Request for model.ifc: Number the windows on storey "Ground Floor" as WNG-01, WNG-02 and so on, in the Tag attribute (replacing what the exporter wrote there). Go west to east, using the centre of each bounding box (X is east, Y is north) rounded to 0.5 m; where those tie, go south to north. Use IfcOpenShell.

First a look at what the model holds.

```python
import ifcopenshell
import ifcopenshell.util.element
import ifcopenshell.util.placement

model = ifcopenshell.open("model.ifc")
print(model.schema)
storey = next(s for s in model.by_type("IfcBuildingStorey") if s.Name == "Ground Floor")
windows = [e for e in ifcopenshell.util.element.get_decomposition(storey) if e.is_a("IfcWindow")]
for e in sorted(windows, key=lambda e: e.id()):
    origin = ifcopenshell.util.placement.get_local_placement(e.ObjectPlacement)[:3, 3]
    print(e.id(), e.Tag, e.Name, origin.round(2) + 0.0, sep=" | ")
```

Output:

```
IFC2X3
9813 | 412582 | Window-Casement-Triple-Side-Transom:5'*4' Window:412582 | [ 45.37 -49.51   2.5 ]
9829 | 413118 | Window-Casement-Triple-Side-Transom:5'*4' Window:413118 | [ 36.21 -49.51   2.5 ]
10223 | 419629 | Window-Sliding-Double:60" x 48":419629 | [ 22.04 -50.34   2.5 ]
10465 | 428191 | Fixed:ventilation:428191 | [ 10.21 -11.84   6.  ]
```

```python
import ifcopenshell
import ifcopenshell.geom
import ifcopenshell.util.element
import ifcopenshell.util.shape

model = ifcopenshell.open("model.ifc")
settings = ifcopenshell.geom.settings()
settings.set("use-world-coords", True)


def centre(element):
    shape = ifcopenshell.geom.create_shape(settings, element)
    return ifcopenshell.util.shape.get_bbox_centroid(shape.geometry)


storey = next(s for s in model.by_type("IfcBuildingStorey") if s.Name == "Ground Floor")
windows = [e for e in ifcopenshell.util.element.get_decomposition(storey) if e.is_a("IfcWindow")]

# Insertion points can sit at a corner or the storey origin, so sort by the geometry (in metres).
centres = {e: centre(e) for e in windows}
windows.sort(key=lambda e: (round(centres[e][0] / 0.5), centres[e][1]))

for i, e in enumerate(windows, start=1):
    number = f"WNG-{i:02d}"
    e.Tag = number
    print(e.id(), number)

model.write("model_rev.ifc")
```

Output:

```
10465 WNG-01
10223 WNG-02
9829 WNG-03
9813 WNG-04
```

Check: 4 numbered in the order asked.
